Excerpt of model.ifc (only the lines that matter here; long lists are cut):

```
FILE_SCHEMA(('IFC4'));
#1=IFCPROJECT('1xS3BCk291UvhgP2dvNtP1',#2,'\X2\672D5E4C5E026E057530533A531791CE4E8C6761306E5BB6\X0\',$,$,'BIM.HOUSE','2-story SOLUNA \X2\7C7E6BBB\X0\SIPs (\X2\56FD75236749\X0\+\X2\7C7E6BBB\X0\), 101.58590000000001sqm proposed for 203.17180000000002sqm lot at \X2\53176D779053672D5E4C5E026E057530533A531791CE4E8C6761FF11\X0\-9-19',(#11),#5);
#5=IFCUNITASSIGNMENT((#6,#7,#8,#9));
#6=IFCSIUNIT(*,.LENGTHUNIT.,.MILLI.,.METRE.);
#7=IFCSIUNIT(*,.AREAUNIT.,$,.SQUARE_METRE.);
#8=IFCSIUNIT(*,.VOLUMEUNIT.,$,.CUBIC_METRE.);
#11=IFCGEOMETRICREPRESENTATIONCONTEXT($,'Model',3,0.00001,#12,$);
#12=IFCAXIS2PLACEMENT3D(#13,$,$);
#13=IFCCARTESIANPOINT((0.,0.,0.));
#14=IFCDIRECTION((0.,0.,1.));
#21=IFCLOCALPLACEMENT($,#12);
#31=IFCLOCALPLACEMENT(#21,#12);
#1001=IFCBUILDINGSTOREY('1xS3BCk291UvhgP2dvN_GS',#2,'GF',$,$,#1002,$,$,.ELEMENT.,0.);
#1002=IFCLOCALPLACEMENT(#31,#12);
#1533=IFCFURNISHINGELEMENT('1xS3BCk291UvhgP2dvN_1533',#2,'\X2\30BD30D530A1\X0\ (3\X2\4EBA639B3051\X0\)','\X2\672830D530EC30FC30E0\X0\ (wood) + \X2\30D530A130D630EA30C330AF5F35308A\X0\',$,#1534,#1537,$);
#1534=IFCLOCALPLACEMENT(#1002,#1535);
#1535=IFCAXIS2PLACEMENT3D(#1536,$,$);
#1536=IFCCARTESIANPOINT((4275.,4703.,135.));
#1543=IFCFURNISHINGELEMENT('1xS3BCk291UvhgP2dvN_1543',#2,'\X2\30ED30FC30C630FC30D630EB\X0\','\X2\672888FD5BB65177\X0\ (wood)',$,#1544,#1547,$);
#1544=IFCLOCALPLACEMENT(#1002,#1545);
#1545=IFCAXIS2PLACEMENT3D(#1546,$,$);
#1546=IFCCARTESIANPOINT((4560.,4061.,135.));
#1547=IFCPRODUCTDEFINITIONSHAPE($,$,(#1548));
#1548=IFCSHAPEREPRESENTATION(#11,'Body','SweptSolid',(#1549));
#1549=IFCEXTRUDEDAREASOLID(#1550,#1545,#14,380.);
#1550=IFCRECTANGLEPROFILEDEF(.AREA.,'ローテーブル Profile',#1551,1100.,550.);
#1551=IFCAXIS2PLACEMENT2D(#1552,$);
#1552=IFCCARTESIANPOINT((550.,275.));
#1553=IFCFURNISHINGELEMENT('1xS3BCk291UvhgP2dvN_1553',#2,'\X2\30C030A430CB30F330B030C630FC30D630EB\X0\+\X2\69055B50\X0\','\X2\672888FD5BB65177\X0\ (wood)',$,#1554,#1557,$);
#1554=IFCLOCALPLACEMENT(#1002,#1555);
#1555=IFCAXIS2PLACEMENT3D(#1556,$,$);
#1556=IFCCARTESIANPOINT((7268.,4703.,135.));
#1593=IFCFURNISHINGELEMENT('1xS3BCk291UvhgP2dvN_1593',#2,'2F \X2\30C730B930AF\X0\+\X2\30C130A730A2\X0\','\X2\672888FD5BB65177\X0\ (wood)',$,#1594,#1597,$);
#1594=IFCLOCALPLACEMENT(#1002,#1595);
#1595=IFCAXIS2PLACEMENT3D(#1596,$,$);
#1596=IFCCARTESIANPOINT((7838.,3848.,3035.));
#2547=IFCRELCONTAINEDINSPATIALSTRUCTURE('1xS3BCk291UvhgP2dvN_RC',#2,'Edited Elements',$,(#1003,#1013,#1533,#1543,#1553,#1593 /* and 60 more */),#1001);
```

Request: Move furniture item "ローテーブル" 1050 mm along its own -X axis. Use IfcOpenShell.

```python
import ifcopenshell
import ifcopenshell.api.geometry
import ifcopenshell.util.placement
import ifcopenshell.util.unit

model = ifcopenshell.open("model.ifc")
unit_scale = ifcopenshell.util.unit.calculate_unit_scale(model)

item = model.by_guid("1xS3BCk291UvhgP2dvN_1543")
matrix = ifcopenshell.util.placement.get_local_placement(item.ObjectPlacement)
matrix[:3, 3] -= matrix[:3, 0] * 1.05 / unit_scale
ifcopenshell.api.geometry.edit_object_placement(model, product=item, matrix=matrix, is_si=False)

print(ifcopenshell.util.placement.get_local_placement(item.ObjectPlacement).round(3) + 0.0)

model.write("model_updated.ifc")
```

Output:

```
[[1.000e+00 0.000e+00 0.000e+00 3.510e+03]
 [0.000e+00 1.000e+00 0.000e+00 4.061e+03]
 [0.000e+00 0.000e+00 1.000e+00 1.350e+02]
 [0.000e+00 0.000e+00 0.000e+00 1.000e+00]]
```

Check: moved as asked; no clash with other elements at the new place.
